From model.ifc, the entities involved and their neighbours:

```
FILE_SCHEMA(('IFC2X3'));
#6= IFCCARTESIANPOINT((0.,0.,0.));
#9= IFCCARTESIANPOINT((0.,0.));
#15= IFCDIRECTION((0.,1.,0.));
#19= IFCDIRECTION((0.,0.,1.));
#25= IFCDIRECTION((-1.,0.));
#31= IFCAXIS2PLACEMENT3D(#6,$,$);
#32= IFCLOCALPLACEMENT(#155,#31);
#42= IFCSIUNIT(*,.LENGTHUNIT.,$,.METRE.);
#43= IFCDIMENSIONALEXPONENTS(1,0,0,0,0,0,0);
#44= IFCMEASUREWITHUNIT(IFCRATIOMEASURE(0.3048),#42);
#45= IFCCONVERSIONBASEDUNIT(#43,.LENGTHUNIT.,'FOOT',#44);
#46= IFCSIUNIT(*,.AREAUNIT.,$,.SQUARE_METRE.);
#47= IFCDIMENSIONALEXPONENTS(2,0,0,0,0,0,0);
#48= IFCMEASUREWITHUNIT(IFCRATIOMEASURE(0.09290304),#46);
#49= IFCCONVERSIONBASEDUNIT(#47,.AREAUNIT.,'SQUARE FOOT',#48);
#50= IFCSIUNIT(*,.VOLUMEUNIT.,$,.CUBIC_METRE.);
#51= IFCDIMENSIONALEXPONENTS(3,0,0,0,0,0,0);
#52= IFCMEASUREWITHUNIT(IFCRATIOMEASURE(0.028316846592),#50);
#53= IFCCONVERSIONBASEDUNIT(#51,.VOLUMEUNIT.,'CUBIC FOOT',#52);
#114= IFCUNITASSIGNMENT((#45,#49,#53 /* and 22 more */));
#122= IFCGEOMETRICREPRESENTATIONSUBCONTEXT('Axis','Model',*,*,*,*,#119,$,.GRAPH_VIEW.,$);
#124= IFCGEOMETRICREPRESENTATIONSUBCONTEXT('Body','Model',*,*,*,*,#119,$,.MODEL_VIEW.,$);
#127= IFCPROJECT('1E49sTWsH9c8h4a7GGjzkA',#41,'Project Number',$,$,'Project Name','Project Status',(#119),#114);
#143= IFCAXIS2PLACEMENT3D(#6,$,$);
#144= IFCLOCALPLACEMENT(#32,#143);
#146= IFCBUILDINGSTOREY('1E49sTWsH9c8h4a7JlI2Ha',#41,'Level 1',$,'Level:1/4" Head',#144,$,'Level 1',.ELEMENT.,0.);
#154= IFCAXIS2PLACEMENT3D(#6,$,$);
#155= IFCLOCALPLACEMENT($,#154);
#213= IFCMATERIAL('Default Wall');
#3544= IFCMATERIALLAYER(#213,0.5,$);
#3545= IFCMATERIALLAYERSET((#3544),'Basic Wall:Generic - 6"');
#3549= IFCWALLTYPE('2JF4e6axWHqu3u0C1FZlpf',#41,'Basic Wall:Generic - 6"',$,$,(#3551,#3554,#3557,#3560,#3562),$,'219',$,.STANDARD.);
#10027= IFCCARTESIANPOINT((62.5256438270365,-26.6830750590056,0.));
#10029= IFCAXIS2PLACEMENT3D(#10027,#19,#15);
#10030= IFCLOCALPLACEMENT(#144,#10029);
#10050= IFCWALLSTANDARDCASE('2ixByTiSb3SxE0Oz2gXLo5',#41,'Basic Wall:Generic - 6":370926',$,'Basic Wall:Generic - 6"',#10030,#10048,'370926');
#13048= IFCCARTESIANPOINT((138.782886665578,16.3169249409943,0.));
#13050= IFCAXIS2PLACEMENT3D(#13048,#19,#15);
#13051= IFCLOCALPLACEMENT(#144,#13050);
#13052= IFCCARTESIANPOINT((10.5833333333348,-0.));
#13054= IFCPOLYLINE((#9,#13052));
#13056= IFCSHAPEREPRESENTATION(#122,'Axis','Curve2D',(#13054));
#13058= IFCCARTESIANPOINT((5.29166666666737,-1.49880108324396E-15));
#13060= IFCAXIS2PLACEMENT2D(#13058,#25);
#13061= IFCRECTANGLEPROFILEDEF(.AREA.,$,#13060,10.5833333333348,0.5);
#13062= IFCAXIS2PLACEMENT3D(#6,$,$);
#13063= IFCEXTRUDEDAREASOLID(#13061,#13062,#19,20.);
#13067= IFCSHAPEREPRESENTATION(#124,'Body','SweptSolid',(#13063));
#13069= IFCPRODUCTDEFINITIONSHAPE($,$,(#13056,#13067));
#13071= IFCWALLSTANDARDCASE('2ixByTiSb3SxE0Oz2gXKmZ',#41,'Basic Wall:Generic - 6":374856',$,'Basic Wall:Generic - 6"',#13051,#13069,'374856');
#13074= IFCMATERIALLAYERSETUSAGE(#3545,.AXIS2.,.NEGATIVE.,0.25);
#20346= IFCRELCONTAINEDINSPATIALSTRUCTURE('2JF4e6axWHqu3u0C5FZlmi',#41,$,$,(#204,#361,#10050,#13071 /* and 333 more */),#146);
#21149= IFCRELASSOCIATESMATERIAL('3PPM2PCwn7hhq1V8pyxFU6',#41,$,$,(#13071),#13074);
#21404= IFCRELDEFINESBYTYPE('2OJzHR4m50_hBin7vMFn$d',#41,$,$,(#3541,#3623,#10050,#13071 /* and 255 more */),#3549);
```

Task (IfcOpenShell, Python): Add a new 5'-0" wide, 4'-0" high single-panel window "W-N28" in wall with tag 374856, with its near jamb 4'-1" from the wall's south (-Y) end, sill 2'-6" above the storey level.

```python
import numpy as np
import ifcopenshell
import ifcopenshell.api.feature
import ifcopenshell.api.geometry
import ifcopenshell.api.root
import ifcopenshell.api.spatial
import ifcopenshell.api.type
import ifcopenshell.geom
import ifcopenshell.util.element
import ifcopenshell.util.placement
import ifcopenshell.util.representation
import ifcopenshell.util.shape
import ifcopenshell.util.unit

model = ifcopenshell.open("model.ifc")
unit_scale = ifcopenshell.util.unit.calculate_unit_scale(model)
settings = ifcopenshell.geom.settings()


def volume(element):
    """Net volume in cubic metres, openings subtracted."""
    shape = ifcopenshell.geom.create_shape(settings, element)
    return ifcopenshell.util.shape.get_volume(shape.geometry)


wall = model.by_guid("2ixByTiSb3SxE0Oz2gXKmZ")
storey = ifcopenshell.util.element.get_container(wall, ifc_class="IfcBuildingStorey")
context = ifcopenshell.util.representation.get_context(model, "Model", "Body", "MODEL_VIEW")
before = volume(wall)

width, height, from_end, sill = 1.524, 1.2192, 1.2446, 0.762  # metres

# The wall runs along its own X axis, and the end named is its -X end.
wall_shape = ifcopenshell.geom.create_shape(settings, wall)
x, y, z = ifcopenshell.util.shape.get_vertices(wall_shape.geometry).T
start = x.min() + from_end
face, thickness = float(y.min()), float(y.max() - y.min())
wall_matrix = ifcopenshell.util.placement.get_local_placement(wall.ObjectPlacement)
level = ifcopenshell.util.placement.get_local_placement(storey.ObjectPlacement)[2, 3]


def in_wall(x, y):
    """Placement at x, y metres in the wall's axes, at sill height."""
    matrix = wall_matrix.copy()
    matrix[:, 3] = wall_matrix @ np.array([x / unit_scale, y / unit_scale, 0.0, 1.0])
    matrix[2, 3] = level + sill / unit_scale
    return matrix


# Opening: a box that overshoots both wall faces by 50 mm.
opening = ifcopenshell.api.root.create_entity(model, ifc_class="IfcOpeningElement")
box = ifcopenshell.api.geometry.add_wall_representation(
    model, context=context, length=width, height=height, thickness=thickness + 0.1
)
ifcopenshell.api.geometry.assign_representation(model, product=opening, representation=box)
ifcopenshell.api.geometry.edit_object_placement(model, product=opening, matrix=in_wall(start, face - 0.05), is_si=False)
ifcopenshell.api.feature.add_feature(model, feature=opening, element=wall)

window = ifcopenshell.api.root.create_entity(model, ifc_class="IfcWindow", name="W-N28")
window.OverallWidth, window.OverallHeight = width / unit_scale, height / unit_scale
body = ifcopenshell.api.geometry.add_window_representation(
    model,
    context=context,
    overall_width=window.OverallWidth,
    overall_height=window.OverallHeight,
    partition_type="SINGLE_PANEL",
)
ifcopenshell.api.geometry.assign_representation(model, product=window, representation=body)
ifcopenshell.api.spatial.assign_container(model, products=[window], relating_structure=storey)
fills = ifcopenshell.api.feature.add_filling(model, opening=opening, element=window)
fills.OwnerHistory = window.OwnerHistory  # required in IFC2X3

# IFC2X3 keeps the operation on the window style.
style = ifcopenshell.api.root.create_entity(model, ifc_class="IfcWindowStyle", name="W-N28")
style.OperationType, style.ConstructionType = "SINGLE_PANEL", "NOTDEFINED"
style.ParameterTakesPrecedence = style.Sizeable = False
ifcopenshell.api.type.assign_type(model, related_objects=[window], relating_type=style)

# Centre the window in the wall's thickness.
ifcopenshell.api.geometry.edit_object_placement(model, product=window, matrix=in_wall(start, face), is_si=False)
window_shape = ifcopenshell.geom.create_shape(settings, window)
depth = ifcopenshell.util.shape.get_vertices(window_shape.geometry)[:, 1]
offset = face + thickness / 2 - (depth.min() + depth.max()) / 2
ifcopenshell.api.geometry.edit_object_placement(model, product=window, matrix=in_wall(start, offset), is_si=False)

after = volume(wall)

print(f"wall volume {before:.3f} -> {after:.3f} m3")

model.write("model_edited.ifc")
```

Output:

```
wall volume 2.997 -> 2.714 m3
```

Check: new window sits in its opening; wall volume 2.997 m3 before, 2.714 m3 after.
